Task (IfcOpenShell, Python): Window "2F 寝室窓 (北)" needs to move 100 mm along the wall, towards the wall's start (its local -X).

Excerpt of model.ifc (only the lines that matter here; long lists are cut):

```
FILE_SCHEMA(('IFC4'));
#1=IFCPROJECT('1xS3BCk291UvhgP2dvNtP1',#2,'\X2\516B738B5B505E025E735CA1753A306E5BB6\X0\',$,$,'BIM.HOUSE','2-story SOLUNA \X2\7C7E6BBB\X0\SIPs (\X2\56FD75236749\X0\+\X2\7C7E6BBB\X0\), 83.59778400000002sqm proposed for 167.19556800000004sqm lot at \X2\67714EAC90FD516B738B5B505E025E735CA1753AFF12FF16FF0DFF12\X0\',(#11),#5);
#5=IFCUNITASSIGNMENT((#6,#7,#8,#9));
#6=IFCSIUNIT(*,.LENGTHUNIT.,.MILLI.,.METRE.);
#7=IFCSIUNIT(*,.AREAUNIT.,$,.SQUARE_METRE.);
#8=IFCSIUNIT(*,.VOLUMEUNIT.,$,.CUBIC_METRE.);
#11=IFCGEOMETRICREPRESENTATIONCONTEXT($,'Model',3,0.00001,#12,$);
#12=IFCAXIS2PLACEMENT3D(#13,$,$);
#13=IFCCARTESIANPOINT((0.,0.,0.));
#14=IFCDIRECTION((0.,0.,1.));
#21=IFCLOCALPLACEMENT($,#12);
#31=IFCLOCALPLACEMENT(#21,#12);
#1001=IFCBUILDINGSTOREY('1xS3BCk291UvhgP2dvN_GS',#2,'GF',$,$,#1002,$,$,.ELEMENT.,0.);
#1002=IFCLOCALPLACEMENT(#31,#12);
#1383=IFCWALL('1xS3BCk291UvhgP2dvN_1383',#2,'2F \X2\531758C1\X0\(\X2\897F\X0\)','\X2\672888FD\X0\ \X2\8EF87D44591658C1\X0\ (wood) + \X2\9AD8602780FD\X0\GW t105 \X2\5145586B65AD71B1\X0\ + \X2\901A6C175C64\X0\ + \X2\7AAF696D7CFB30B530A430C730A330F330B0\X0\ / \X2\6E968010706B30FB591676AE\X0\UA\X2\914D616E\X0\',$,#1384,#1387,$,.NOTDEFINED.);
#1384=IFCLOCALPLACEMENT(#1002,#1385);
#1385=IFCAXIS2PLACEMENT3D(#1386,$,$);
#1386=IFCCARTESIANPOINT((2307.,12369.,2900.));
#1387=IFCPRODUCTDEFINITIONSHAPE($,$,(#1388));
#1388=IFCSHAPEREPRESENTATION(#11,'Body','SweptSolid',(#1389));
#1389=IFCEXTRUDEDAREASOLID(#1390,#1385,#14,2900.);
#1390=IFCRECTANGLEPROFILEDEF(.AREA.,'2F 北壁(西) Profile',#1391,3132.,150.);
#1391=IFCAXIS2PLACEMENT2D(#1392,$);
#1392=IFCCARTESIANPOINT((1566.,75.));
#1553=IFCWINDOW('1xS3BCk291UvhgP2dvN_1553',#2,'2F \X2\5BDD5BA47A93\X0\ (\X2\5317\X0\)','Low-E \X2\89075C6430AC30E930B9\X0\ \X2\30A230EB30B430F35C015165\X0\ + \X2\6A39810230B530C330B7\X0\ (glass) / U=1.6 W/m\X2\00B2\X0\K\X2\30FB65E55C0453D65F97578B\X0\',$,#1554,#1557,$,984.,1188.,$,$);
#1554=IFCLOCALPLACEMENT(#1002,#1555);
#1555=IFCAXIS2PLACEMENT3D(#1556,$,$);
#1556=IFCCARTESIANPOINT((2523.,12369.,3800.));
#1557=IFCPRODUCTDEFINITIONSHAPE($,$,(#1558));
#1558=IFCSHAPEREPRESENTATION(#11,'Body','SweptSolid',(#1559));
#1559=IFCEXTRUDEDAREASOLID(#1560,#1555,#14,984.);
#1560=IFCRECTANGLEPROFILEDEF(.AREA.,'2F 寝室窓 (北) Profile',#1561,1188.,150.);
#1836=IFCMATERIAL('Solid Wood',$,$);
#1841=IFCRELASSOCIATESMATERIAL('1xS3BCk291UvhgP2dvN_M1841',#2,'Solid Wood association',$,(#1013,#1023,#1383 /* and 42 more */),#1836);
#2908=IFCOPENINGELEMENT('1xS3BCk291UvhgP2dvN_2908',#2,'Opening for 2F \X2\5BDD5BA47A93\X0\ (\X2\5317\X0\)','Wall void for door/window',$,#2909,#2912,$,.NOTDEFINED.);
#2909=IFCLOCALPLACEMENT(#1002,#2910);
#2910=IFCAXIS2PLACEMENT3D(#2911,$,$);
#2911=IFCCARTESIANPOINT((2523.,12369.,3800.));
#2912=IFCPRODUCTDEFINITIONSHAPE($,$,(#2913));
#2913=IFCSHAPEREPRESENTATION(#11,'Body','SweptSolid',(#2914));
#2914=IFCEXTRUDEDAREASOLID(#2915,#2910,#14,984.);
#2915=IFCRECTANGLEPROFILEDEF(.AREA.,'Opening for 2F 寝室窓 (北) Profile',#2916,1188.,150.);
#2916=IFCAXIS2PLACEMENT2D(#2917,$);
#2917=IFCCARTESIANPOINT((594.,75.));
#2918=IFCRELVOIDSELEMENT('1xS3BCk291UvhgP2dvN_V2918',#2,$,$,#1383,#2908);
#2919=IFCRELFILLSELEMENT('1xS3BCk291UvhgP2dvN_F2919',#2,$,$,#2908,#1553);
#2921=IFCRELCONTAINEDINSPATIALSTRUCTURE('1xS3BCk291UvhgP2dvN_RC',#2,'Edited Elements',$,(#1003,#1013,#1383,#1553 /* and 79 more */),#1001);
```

```python
import ifcopenshell
import ifcopenshell.api.geometry
import ifcopenshell.util.placement

model = ifcopenshell.open("model.ifc")

window = model.by_guid("1xS3BCk291UvhgP2dvN_1553")
opening = window.FillsVoids[0].RelatingOpeningElement
wall = opening.VoidsElements[0].RelatingBuildingElement

wall_matrix = ifcopenshell.util.placement.get_local_placement(wall.ObjectPlacement)
shift = wall_matrix[:3, 0] * -100.0
before = ifcopenshell.util.placement.get_local_placement(window.ObjectPlacement)[:3, 3].copy()

# The window is not placed relative to its opening, so move both.
for product in (opening, window):
    matrix = ifcopenshell.util.placement.get_local_placement(product.ObjectPlacement)
    matrix[:3, 3] += shift
    ifcopenshell.api.geometry.edit_object_placement(model, product=product, matrix=matrix, is_si=False)

after = ifcopenshell.util.placement.get_local_placement(window.ObjectPlacement)[:3, 3]
print("window moved by", (after - before).round(3) + 0.0)

model.write("model_updated.ifc")
```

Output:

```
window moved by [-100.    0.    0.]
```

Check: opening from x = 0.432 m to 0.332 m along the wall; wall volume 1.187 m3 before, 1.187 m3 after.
